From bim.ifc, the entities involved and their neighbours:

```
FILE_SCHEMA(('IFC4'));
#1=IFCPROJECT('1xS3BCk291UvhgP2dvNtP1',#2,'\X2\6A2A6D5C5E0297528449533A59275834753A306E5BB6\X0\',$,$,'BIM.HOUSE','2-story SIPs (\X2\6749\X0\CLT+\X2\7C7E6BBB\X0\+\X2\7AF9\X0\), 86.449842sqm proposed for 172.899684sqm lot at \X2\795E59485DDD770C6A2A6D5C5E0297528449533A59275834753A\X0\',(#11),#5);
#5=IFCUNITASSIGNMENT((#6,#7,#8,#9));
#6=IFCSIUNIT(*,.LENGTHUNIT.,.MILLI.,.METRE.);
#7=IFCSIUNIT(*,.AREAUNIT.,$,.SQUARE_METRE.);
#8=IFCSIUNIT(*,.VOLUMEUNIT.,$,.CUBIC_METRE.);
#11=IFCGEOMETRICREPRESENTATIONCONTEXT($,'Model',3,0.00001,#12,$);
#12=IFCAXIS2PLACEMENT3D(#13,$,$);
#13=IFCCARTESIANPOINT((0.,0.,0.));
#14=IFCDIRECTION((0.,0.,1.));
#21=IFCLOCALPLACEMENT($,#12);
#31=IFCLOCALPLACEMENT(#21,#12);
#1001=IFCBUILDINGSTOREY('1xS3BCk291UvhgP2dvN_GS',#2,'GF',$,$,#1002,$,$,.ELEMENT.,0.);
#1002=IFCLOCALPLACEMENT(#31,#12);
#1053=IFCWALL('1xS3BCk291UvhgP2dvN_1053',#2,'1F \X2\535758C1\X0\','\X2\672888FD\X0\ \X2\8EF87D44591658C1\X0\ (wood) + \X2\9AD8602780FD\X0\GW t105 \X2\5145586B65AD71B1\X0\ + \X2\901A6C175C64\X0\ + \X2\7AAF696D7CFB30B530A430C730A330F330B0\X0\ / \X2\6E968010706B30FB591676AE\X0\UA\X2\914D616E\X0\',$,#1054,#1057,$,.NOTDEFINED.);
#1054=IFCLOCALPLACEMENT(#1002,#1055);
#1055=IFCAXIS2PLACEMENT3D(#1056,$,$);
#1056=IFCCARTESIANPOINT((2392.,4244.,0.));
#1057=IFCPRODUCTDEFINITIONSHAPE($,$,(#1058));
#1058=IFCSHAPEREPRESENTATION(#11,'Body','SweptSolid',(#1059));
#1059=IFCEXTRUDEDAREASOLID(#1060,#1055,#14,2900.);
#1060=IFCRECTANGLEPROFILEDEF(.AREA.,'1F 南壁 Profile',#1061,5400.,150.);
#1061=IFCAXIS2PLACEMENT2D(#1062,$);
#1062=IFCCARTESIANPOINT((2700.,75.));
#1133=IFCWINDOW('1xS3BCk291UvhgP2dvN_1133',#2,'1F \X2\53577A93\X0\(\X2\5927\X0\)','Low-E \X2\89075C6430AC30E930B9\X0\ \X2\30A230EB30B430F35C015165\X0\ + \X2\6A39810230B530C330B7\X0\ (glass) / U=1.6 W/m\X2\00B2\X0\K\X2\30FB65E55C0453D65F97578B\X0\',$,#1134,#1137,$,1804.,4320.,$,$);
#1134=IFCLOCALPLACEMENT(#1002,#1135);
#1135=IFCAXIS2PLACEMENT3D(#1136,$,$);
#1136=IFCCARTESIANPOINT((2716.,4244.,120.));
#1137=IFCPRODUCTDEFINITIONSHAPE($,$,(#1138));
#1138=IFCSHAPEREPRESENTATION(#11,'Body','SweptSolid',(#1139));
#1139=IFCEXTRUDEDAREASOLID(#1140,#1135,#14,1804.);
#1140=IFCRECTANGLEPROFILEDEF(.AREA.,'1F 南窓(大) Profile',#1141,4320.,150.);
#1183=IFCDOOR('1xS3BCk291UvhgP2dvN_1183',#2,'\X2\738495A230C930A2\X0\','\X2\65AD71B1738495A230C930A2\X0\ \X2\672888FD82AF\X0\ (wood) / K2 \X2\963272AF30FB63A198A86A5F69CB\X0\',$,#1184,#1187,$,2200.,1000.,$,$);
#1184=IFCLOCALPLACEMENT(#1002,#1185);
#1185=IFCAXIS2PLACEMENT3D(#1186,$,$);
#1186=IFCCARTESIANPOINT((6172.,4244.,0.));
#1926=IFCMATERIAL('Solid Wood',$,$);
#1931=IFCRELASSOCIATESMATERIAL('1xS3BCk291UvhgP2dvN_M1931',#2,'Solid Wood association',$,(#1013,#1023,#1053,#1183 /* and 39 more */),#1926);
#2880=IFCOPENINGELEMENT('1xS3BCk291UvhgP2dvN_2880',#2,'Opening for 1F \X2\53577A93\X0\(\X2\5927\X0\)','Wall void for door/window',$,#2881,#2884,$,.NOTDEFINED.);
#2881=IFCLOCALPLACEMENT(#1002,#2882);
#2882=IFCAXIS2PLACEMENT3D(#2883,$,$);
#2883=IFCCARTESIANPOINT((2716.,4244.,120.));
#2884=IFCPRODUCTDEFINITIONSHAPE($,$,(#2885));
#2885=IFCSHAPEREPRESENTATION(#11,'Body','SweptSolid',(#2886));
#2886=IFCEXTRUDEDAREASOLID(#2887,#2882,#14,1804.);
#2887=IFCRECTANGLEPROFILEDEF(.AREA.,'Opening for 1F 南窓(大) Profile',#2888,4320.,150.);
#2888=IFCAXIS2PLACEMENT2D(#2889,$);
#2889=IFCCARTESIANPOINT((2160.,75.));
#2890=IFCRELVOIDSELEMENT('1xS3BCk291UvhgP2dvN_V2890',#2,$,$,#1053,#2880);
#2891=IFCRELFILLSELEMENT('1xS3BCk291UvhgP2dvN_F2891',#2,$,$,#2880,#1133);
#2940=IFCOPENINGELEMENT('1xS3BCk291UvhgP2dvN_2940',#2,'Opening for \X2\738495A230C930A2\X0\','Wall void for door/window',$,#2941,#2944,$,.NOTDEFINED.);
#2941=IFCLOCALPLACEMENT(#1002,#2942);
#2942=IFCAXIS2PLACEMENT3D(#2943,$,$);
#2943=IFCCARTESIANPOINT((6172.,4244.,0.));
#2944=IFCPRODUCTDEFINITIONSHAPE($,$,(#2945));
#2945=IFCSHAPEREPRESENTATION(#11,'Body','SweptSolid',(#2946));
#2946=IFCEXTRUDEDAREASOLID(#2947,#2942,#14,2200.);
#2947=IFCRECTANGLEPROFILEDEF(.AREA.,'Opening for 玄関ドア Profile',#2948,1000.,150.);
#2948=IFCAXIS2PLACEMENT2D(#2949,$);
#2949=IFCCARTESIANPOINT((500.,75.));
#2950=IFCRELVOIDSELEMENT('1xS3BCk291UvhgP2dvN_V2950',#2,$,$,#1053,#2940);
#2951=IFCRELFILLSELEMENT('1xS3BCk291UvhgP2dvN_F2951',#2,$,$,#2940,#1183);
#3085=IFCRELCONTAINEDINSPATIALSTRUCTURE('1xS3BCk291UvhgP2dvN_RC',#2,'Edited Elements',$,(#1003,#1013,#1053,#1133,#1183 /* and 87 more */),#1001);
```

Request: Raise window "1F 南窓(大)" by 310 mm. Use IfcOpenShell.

```python
import numpy as np
import ifcopenshell
import ifcopenshell.api.geometry
import ifcopenshell.util.placement
import ifcopenshell.util.unit

model = ifcopenshell.open("bim.ifc")
unit_scale = ifcopenshell.util.unit.calculate_unit_scale(model)

window = model.by_guid("1xS3BCk291UvhgP2dvN_1133")
opening = window.FillsVoids[0].RelatingOpeningElement
dz = 0.31 / unit_scale

shift = np.array([0.0, 0.0, dz])
# The window is not placed relative to its opening, so move both.
for product in (opening, window):
    matrix = ifcopenshell.util.placement.get_local_placement(product.ObjectPlacement)
    matrix[:3, 3] += shift
    ifcopenshell.api.geometry.edit_object_placement(model, product=product, matrix=matrix, is_si=False)

print(f"moved by {dz * unit_scale:+.3f} m")

model.write("bim_edited.ifc")
```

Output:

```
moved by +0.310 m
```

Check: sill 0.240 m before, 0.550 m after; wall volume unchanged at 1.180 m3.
